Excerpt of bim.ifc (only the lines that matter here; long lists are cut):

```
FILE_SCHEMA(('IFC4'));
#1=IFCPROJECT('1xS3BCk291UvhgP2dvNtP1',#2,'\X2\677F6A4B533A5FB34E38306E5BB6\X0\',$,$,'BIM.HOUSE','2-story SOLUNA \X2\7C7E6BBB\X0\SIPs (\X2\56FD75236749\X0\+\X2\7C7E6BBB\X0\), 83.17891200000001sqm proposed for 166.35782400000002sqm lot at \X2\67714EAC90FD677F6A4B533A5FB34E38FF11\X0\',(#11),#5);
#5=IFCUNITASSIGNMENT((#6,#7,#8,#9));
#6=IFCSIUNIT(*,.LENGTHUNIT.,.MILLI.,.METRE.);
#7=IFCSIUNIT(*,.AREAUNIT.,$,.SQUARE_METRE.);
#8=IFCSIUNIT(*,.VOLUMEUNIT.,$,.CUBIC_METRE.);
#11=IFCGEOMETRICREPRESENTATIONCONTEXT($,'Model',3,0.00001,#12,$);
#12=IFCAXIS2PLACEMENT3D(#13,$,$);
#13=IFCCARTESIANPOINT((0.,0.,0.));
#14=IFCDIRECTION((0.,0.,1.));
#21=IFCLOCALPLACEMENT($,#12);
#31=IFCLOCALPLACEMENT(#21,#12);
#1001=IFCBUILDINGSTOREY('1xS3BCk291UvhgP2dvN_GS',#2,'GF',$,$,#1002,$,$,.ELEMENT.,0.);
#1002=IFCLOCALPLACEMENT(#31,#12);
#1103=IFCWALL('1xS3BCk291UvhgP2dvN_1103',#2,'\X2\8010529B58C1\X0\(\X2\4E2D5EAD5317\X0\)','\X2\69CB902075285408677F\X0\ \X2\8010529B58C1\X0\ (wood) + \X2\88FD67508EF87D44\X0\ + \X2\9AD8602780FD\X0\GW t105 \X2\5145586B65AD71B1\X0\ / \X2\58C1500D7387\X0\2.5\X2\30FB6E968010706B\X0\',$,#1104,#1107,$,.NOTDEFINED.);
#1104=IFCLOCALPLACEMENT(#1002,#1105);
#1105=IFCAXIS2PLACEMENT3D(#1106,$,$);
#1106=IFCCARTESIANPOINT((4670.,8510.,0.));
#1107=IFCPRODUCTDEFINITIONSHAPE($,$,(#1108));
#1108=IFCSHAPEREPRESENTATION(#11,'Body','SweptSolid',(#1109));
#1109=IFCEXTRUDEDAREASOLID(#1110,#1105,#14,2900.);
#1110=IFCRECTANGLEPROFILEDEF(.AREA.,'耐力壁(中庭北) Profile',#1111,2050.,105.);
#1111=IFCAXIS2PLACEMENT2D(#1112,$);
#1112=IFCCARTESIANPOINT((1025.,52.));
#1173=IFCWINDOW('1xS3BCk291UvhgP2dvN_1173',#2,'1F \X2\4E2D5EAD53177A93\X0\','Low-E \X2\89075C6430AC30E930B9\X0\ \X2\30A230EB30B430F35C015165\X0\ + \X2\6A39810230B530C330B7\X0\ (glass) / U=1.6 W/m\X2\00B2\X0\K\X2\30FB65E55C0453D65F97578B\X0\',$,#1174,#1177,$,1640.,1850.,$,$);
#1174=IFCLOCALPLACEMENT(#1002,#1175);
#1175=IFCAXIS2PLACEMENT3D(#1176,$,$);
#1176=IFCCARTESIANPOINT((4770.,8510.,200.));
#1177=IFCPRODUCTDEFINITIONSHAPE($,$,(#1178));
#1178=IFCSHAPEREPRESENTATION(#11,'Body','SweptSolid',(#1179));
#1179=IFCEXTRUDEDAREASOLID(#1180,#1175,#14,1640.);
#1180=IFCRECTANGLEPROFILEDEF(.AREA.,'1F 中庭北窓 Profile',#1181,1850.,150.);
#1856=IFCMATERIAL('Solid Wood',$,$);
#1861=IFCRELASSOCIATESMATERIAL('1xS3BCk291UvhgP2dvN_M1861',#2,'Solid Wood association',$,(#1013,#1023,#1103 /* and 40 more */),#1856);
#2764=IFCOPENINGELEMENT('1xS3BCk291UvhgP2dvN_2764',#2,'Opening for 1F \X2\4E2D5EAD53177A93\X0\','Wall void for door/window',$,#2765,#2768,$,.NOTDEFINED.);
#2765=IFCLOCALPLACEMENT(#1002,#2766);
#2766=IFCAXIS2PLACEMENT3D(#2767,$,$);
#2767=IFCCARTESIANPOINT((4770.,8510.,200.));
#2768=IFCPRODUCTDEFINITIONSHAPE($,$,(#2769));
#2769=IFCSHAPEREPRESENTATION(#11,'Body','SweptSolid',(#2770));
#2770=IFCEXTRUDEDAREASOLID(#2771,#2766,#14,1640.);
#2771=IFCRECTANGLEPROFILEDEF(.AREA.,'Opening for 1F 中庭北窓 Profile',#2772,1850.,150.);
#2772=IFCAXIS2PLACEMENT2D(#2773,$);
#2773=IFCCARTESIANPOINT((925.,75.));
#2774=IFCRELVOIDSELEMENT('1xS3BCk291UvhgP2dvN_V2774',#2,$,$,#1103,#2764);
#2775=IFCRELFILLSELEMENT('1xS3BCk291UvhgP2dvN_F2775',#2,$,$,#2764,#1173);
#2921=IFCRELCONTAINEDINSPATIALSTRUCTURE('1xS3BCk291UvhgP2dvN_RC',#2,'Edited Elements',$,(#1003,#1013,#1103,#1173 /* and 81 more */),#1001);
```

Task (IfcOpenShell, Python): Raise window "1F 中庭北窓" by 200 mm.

```python
import numpy as np
import ifcopenshell
import ifcopenshell.api.geometry
import ifcopenshell.util.placement
import ifcopenshell.util.unit

model = ifcopenshell.open("bim.ifc")
unit_scale = ifcopenshell.util.unit.calculate_unit_scale(model)

window = model.by_guid("1xS3BCk291UvhgP2dvN_1173")
opening = window.FillsVoids[0].RelatingOpeningElement
dz = 0.2 / unit_scale

shift = np.array([0.0, 0.0, dz])
# The window is not placed relative to its opening, so move both.
for product in (opening, window):
    matrix = ifcopenshell.util.placement.get_local_placement(product.ObjectPlacement)
    matrix[:3, 3] += shift
    ifcopenshell.api.geometry.edit_object_placement(model, product=product, matrix=matrix, is_si=False)

print(f"moved by {dz * unit_scale:+.3f} m")

model.write("bim_rev.ifc")
```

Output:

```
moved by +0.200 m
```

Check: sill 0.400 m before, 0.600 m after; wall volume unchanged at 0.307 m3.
